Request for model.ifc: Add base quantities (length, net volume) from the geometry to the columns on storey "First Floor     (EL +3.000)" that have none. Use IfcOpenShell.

First a look at what the model holds.

```python
import ifcopenshell
import ifcopenshell.util.element
import ifcopenshell.util.unit

model = ifcopenshell.open("model.ifc")
print(model.schema)
for unit_type in ("LENGTHUNIT", "AREAUNIT", "VOLUMEUNIT"):
    print(unit_type, ifcopenshell.util.unit.calculate_unit_scale(model, unit_type))
storey = next(s for s in model.by_type("IfcBuildingStorey") if s.Name == "First Floor     (EL +3.000)")
columns = [e for e in ifcopenshell.util.element.get_decomposition(storey) if e.is_a("IfcColumn")]
for e in sorted(columns, key=lambda e: e.id()):
    print(e.id(), e.is_a(), e.Name, list(ifcopenshell.util.element.get_psets(e, qtos_only=True)), sep=" | ")
```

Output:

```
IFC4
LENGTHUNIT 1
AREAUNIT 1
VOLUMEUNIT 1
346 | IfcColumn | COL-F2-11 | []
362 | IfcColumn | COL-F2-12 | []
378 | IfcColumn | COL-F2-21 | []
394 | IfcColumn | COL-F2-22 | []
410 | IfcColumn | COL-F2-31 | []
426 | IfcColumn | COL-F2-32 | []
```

```python
import ifcopenshell
import ifcopenshell.api.pset
import ifcopenshell.geom
import ifcopenshell.util.element
import ifcopenshell.util.shape
import ifcopenshell.util.unit

model = ifcopenshell.open("model.ifc")
unit_scale = ifcopenshell.util.unit.calculate_unit_scale(model)
volume_scale = ifcopenshell.util.unit.calculate_unit_scale(model, "VOLUMEUNIT")
settings = ifcopenshell.geom.settings()

storey = next(s for s in model.by_type("IfcBuildingStorey") if s.Name == "First Floor     (EL +3.000)")
columns = [e for e in ifcopenshell.util.element.get_decomposition(storey) if e.is_a("IfcColumn")]

for e in sorted(columns, key=lambda e: e.id()):
    if ifcopenshell.util.element.get_psets(e, qtos_only=True, should_inherit=False):
        continue
    # Geometry comes back in metres, in the element's own axes.
    shape = ifcopenshell.geom.create_shape(settings, e)
    values = {
        "Length": ifcopenshell.util.shape.get_z(shape.geometry) / unit_scale,
        "NetVolume": ifcopenshell.util.shape.get_volume(shape.geometry) / volume_scale,
    }
    qto = ifcopenshell.api.pset.add_qto(model, product=e, name="Qto_ColumnBaseQuantities")
    ifcopenshell.api.pset.edit_qto(model, qto=qto, properties=values)
    print(e.id(), {k: round(v, 3) for k, v in values.items()})

model.write("model-out.ifc")
```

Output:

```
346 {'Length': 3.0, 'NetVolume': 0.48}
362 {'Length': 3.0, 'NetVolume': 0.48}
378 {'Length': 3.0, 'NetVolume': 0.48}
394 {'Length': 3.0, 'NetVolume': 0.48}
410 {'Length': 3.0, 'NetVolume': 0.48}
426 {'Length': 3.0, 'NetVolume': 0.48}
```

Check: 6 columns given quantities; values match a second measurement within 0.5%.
